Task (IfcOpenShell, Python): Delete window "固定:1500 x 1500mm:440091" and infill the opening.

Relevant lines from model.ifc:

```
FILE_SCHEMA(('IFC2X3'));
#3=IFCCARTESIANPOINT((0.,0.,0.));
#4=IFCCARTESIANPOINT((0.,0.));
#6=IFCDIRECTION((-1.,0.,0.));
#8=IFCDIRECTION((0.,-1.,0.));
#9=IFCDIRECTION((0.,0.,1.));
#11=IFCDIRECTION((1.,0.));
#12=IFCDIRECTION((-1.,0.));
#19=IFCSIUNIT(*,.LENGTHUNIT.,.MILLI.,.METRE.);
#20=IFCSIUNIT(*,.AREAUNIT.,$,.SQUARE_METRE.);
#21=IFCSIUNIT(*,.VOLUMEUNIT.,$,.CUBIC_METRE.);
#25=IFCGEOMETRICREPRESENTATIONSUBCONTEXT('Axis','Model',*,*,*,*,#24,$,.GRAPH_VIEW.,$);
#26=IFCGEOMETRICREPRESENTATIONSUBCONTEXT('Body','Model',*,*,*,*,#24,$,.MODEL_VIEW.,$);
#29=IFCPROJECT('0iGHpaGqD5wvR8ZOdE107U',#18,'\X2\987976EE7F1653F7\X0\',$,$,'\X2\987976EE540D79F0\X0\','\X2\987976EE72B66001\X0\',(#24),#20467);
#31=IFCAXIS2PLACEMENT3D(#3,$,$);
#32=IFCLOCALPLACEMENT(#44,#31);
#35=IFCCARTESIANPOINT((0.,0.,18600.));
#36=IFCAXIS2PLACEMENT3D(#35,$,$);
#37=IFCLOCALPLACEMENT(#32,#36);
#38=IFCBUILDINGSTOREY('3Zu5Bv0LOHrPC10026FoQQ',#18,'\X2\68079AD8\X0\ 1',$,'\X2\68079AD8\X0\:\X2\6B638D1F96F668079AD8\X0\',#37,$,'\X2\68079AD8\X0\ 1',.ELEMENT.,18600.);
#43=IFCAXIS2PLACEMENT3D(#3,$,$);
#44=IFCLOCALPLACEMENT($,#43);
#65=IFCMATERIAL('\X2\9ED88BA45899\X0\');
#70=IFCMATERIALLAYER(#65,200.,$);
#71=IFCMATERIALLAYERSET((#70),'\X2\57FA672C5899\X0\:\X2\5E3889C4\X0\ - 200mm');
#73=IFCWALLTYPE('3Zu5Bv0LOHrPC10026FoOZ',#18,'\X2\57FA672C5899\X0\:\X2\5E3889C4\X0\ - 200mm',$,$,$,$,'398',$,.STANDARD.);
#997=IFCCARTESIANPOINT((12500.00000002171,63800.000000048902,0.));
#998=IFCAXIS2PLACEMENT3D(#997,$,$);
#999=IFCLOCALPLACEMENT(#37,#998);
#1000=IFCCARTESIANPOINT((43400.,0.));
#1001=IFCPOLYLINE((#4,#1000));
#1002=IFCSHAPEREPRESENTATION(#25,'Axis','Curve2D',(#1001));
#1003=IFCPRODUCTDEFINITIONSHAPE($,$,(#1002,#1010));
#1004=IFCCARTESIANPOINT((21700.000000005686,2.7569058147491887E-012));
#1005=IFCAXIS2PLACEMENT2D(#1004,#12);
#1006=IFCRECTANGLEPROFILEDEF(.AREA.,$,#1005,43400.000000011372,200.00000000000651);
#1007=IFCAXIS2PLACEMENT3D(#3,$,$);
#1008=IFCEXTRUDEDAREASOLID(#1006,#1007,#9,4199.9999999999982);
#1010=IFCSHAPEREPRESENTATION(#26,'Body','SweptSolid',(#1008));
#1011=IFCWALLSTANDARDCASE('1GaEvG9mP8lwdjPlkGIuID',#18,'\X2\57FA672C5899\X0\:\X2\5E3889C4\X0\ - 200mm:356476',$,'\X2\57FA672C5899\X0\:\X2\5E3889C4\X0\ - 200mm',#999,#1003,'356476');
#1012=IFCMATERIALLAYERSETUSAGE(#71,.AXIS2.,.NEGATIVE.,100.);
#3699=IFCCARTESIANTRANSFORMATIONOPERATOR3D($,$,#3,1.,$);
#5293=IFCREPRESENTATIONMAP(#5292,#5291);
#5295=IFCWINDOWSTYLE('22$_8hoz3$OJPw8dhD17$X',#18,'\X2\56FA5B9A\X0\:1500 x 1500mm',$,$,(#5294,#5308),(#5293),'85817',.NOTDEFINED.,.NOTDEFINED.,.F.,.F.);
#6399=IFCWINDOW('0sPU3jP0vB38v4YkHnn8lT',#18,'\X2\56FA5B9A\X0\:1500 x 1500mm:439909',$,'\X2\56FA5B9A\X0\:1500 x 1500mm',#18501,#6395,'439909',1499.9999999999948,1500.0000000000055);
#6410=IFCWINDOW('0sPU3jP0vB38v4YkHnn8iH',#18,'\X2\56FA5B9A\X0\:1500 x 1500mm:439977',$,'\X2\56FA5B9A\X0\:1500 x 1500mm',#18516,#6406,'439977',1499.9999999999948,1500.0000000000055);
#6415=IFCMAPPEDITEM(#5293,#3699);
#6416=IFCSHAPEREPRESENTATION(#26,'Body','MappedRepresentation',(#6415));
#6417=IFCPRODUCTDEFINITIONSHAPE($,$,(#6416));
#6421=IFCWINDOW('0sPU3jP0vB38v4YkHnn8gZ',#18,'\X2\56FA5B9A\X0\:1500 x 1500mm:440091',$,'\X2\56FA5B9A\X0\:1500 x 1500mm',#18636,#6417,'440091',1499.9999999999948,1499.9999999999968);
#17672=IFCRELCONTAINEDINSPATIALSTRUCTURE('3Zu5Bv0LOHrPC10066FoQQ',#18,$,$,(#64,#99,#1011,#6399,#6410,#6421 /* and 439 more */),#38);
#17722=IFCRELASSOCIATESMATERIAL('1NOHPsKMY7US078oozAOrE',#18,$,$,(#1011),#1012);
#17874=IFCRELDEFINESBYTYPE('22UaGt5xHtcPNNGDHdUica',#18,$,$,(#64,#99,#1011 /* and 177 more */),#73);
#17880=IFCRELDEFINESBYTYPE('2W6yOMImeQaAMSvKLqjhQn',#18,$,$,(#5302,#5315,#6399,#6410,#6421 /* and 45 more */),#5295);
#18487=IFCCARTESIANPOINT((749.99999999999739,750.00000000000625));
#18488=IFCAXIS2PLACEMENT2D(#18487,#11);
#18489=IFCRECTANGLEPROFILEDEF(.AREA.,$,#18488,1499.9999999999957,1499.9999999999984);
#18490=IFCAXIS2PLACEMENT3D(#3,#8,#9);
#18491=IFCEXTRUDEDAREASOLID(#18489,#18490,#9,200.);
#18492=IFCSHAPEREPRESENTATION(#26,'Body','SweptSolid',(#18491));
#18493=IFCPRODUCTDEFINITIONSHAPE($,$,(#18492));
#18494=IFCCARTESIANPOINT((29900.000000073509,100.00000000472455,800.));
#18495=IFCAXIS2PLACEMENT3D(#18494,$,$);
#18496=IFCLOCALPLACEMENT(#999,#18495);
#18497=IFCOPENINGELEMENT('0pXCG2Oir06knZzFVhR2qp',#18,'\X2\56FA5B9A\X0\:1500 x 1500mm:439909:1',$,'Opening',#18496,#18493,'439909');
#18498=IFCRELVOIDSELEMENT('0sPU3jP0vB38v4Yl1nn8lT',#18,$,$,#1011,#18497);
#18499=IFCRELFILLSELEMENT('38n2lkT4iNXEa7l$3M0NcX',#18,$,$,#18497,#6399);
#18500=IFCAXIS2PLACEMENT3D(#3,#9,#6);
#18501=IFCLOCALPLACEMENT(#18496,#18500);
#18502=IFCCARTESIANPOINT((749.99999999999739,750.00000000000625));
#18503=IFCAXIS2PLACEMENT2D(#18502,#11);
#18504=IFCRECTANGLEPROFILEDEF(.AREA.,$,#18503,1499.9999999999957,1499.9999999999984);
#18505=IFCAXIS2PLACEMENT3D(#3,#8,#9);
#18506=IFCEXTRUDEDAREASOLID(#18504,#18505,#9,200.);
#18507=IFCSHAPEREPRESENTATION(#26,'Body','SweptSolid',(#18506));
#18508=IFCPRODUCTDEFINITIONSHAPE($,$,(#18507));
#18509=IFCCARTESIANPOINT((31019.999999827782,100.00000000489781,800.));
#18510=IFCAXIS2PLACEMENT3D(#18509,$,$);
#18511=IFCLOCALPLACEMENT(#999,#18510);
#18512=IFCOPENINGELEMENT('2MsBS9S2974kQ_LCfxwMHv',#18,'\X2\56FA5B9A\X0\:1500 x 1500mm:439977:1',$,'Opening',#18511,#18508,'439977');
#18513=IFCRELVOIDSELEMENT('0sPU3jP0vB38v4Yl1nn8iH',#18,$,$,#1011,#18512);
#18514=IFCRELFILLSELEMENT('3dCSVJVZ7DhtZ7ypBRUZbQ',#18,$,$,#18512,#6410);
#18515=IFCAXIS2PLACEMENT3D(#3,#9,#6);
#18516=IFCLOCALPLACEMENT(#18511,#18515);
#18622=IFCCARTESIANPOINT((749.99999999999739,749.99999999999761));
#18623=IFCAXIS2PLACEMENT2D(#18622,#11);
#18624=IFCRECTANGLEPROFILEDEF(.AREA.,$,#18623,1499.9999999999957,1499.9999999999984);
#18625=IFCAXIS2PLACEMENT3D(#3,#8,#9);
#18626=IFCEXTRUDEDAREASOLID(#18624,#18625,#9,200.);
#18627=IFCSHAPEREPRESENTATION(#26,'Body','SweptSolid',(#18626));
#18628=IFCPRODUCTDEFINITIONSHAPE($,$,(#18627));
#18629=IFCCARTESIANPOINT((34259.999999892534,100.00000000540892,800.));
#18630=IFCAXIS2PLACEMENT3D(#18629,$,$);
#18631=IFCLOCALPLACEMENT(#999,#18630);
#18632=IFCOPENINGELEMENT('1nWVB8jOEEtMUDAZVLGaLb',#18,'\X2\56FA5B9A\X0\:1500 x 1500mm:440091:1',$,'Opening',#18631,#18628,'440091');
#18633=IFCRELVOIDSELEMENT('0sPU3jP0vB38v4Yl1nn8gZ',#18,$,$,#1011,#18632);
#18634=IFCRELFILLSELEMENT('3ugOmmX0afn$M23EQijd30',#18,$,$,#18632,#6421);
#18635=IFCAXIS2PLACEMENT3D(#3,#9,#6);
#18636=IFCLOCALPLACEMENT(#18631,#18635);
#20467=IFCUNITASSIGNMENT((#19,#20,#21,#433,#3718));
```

```python
import ifcopenshell
import ifcopenshell.api.feature
import ifcopenshell.api.root
import ifcopenshell.geom
import ifcopenshell.util.shape

model = ifcopenshell.open("model.ifc")
settings = ifcopenshell.geom.settings()


def volume(element):
    """Net volume in cubic metres, openings subtracted."""
    shape = ifcopenshell.geom.create_shape(settings, element)
    return ifcopenshell.util.shape.get_volume(shape.geometry)


window = model.by_id(6421)
opening = window.FillsVoids[0].RelatingOpeningElement
wall = opening.VoidsElements[0].RelatingBuildingElement
before = volume(wall)

ifcopenshell.api.root.remove_product(model, product=window)
ifcopenshell.api.feature.remove_feature(model, feature=opening)

after = volume(wall)

print(f"wall volume {before:.3f} -> {after:.3f} m3")

model.write("model_rev.ifc")
```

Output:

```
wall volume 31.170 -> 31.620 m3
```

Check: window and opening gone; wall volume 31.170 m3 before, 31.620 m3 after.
